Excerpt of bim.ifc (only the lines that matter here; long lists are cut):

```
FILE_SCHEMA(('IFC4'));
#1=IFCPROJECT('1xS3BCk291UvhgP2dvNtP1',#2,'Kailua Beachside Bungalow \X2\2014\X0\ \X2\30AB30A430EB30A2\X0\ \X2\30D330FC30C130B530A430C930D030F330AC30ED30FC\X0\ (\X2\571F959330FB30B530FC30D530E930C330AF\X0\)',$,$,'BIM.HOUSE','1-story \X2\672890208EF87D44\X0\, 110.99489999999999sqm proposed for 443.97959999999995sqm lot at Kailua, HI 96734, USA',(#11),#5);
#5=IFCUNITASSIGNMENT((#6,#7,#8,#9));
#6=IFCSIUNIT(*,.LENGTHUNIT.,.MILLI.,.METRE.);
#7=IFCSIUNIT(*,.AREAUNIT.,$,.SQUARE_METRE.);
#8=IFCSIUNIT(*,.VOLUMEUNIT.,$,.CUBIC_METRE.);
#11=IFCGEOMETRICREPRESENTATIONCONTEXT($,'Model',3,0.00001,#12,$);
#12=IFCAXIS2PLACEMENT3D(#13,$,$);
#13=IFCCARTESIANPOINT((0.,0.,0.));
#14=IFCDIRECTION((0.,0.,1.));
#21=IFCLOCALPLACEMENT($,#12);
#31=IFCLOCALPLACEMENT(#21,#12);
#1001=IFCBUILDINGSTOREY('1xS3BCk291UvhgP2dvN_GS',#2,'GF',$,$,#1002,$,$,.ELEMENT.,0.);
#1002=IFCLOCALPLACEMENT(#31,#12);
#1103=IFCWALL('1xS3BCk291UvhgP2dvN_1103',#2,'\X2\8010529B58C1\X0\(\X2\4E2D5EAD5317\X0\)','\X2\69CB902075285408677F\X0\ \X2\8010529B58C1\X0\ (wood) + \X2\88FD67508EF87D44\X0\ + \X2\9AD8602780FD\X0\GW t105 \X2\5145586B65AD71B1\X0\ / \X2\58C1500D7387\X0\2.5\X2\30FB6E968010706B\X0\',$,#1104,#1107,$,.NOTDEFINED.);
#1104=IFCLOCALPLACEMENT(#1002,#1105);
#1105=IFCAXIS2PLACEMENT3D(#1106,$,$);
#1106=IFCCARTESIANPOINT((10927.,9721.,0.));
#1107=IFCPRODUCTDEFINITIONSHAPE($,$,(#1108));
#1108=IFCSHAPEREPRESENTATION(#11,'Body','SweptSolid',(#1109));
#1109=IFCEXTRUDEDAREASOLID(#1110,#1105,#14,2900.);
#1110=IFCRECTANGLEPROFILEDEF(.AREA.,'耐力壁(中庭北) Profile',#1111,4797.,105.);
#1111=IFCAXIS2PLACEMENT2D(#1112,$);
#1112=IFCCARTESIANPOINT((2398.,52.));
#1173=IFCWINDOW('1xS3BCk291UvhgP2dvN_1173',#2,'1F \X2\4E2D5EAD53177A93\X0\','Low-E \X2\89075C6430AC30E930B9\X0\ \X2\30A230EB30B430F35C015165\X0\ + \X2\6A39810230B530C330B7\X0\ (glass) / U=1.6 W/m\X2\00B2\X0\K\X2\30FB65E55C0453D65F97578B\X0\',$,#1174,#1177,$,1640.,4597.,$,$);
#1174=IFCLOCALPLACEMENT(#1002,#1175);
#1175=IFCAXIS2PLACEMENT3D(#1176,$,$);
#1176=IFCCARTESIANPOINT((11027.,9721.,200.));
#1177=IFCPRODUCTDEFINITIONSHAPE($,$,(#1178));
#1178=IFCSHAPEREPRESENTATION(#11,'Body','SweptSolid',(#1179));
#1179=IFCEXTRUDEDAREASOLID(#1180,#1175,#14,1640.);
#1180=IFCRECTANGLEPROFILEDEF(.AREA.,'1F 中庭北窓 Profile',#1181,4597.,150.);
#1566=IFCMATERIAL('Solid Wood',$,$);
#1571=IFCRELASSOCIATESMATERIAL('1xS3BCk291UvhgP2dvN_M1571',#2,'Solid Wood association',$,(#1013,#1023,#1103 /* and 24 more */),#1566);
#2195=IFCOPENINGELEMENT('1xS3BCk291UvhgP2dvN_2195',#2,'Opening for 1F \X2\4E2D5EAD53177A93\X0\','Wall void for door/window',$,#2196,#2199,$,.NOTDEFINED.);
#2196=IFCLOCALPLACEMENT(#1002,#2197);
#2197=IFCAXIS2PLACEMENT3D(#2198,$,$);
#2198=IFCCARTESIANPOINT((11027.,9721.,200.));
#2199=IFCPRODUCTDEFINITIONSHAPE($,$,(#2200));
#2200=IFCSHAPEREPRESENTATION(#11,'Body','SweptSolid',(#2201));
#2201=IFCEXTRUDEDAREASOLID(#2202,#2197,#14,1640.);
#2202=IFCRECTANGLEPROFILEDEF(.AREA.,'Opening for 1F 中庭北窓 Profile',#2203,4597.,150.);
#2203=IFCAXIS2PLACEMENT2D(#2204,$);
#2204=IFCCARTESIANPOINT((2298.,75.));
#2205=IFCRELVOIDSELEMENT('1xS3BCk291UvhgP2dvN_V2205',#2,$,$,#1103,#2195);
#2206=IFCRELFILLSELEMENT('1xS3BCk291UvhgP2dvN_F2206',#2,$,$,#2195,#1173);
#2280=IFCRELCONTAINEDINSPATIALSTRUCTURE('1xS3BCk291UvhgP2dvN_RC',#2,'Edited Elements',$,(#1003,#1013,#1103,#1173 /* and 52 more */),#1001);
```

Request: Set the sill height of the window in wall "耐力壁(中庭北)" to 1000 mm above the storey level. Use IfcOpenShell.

```python
import numpy as np
import ifcopenshell
import ifcopenshell.api.geometry
import ifcopenshell.geom
import ifcopenshell.util.element
import ifcopenshell.util.placement
import ifcopenshell.util.shape
import ifcopenshell.util.unit

model = ifcopenshell.open("bim.ifc")
unit_scale = ifcopenshell.util.unit.calculate_unit_scale(model)

window = model.by_id(1173)
opening = window.FillsVoids[0].RelatingOpeningElement
storey = ifcopenshell.util.element.get_container(window, ifc_class="IfcBuildingStorey")
level = ifcopenshell.util.placement.get_local_placement(storey.ObjectPlacement)[2, 3]

# The opening's origin need not be at the sill, so measure its lowest point.
shape = ifcopenshell.geom.create_shape(ifcopenshell.geom.settings(), opening)
bottom = ifcopenshell.util.shape.get_shape_bottom_elevation(shape, shape.geometry) / unit_scale
dz = level + 1000.0 - bottom

shift = np.array([0.0, 0.0, dz])
# The window is not placed relative to its opening, so move both.
for product in (opening, window):
    matrix = ifcopenshell.util.placement.get_local_placement(product.ObjectPlacement)
    matrix[:3, 3] += shift
    ifcopenshell.api.geometry.edit_object_placement(model, product=product, matrix=matrix, is_si=False)

print(f"moved by {dz * unit_scale:+.3f} m")

model.write("bim_rev.ifc")
```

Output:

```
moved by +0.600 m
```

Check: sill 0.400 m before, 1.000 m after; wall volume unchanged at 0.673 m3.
